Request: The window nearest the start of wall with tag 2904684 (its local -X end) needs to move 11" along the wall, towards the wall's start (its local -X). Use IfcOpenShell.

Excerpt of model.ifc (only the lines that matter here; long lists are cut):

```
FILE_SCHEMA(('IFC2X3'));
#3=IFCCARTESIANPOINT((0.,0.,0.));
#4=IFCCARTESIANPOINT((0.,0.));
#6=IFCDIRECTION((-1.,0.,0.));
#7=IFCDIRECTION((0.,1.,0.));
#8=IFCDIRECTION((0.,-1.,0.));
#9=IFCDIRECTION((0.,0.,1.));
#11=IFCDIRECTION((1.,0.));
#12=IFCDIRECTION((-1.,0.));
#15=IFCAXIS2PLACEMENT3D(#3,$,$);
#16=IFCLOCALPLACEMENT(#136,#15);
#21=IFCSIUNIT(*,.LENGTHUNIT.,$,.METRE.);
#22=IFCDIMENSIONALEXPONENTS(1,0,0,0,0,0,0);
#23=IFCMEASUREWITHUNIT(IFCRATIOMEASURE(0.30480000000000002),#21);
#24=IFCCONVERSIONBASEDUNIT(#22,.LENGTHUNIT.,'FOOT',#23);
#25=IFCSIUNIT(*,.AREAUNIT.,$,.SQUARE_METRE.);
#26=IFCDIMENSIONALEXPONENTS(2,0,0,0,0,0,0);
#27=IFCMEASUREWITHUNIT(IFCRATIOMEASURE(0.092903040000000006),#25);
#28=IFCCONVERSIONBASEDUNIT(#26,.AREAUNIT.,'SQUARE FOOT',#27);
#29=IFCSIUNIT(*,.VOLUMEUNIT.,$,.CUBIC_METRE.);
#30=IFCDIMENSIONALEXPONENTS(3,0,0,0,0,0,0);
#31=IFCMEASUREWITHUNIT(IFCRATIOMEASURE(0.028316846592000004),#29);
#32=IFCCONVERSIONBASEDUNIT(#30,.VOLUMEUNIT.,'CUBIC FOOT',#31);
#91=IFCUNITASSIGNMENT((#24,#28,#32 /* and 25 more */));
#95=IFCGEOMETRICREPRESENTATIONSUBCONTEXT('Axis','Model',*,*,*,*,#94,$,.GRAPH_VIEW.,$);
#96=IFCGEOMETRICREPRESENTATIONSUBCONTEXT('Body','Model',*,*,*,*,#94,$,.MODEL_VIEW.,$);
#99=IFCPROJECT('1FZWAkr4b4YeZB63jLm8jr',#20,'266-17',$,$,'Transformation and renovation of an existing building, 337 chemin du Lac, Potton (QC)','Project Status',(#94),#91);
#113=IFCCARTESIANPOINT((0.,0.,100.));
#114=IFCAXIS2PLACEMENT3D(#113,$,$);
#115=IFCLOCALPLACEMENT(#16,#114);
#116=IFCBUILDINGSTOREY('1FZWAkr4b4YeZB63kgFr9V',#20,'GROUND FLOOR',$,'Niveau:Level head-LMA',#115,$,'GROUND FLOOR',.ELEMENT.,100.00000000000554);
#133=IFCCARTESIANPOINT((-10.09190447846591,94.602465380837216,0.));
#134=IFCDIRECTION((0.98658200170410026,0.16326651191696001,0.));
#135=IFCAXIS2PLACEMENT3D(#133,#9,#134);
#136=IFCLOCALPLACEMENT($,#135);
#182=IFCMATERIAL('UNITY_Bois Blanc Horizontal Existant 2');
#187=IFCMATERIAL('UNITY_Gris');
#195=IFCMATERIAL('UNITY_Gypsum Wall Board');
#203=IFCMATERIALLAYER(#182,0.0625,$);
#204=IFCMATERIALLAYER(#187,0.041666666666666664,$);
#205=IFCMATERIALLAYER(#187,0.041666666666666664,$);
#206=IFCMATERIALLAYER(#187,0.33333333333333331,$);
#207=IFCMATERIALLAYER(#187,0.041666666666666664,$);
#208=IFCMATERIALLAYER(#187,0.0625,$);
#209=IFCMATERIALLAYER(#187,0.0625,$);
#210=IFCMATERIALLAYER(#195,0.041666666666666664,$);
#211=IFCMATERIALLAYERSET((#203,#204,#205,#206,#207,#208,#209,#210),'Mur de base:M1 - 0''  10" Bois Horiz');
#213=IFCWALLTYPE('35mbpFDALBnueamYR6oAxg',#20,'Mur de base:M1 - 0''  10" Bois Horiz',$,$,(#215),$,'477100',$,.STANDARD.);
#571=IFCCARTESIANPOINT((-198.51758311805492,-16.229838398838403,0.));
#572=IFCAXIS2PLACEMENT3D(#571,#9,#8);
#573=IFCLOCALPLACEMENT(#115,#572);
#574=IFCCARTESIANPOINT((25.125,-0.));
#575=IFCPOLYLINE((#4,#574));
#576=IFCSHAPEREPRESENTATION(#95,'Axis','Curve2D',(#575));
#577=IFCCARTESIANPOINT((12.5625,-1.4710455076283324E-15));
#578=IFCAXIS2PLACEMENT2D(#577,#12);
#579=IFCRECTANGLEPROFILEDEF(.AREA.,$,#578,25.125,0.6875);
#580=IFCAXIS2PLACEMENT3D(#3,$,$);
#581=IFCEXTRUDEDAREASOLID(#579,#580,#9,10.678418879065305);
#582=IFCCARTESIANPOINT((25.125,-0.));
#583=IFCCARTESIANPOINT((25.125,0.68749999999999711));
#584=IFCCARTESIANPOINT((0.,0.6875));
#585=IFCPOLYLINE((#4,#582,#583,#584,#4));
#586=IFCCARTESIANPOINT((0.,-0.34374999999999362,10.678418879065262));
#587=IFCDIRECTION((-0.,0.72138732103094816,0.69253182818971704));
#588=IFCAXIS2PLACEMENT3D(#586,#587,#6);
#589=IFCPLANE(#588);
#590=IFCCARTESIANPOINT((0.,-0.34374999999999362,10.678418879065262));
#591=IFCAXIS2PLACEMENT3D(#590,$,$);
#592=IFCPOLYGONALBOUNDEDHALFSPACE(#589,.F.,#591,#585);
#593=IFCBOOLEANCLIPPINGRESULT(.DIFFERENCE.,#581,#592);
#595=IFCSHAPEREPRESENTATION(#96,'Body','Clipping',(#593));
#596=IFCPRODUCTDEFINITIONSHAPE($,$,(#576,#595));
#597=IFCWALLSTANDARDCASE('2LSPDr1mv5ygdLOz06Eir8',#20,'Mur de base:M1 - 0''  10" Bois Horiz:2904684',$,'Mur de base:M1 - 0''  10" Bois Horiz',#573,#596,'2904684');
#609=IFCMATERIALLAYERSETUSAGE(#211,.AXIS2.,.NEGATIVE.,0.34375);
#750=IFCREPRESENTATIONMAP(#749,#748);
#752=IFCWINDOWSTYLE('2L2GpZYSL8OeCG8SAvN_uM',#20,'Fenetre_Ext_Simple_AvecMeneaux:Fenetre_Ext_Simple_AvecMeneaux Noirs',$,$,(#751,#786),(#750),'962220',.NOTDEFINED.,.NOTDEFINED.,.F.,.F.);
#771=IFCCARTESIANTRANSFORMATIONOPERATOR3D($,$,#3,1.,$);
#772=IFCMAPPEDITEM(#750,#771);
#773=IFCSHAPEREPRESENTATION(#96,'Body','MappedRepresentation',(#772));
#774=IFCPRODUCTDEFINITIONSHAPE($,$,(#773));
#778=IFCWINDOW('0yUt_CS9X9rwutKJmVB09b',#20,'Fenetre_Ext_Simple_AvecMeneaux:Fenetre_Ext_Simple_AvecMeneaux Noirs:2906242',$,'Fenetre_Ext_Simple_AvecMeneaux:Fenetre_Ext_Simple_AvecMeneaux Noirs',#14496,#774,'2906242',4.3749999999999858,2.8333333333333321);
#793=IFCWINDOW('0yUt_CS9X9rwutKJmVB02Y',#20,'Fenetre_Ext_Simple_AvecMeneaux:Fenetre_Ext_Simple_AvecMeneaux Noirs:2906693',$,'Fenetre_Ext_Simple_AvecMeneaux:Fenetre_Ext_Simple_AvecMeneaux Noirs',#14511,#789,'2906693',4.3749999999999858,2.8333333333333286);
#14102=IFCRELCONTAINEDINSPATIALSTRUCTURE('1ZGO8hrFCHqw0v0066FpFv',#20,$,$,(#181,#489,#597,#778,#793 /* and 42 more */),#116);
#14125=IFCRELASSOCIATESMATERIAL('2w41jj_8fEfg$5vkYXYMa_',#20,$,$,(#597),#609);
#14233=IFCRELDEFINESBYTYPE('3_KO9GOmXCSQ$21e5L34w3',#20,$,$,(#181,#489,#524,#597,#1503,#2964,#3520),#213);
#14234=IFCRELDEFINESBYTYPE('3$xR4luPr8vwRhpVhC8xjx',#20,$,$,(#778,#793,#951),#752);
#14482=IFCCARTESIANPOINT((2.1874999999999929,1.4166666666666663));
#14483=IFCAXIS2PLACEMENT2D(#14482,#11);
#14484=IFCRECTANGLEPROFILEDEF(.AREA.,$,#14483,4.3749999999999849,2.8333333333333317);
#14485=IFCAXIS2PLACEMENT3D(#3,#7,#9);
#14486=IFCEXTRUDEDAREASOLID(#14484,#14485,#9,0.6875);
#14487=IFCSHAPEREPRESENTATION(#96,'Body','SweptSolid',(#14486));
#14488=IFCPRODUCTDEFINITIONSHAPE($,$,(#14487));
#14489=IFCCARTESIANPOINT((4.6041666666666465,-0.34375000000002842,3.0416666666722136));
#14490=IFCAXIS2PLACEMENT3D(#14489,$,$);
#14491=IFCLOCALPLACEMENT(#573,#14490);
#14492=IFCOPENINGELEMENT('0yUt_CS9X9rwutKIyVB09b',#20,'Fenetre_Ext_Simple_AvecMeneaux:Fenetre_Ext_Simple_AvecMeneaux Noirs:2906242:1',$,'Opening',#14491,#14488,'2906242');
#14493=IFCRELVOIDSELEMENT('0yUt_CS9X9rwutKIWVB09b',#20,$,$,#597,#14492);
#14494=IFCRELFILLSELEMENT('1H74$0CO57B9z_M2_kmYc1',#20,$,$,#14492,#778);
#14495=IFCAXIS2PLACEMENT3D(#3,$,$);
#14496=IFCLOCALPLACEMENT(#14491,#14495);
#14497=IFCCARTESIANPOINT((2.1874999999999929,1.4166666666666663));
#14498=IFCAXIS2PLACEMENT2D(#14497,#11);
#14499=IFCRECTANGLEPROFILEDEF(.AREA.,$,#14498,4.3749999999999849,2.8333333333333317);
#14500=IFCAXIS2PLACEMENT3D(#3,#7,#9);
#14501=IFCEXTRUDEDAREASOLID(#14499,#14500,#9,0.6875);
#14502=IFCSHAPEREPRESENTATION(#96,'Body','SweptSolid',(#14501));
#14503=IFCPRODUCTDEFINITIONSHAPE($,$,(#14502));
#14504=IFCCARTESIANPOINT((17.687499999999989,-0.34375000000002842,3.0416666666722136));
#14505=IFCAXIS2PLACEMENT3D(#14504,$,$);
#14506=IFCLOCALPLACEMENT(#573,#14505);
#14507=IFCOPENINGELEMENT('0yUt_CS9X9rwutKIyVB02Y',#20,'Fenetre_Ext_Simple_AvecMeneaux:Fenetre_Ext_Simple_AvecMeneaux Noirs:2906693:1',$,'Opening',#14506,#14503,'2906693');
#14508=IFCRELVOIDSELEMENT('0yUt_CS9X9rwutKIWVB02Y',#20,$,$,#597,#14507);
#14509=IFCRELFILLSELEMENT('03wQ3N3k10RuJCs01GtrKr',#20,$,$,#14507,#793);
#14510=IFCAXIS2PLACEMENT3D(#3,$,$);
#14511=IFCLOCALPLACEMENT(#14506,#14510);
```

```python
import ifcopenshell
import ifcopenshell.api.geometry
import ifcopenshell.util.placement
import ifcopenshell.util.unit

model = ifcopenshell.open("model.ifc")
unit_scale = ifcopenshell.util.unit.calculate_unit_scale(model)

window = model.by_id(778)
opening = window.FillsVoids[0].RelatingOpeningElement
wall = opening.VoidsElements[0].RelatingBuildingElement

wall_matrix = ifcopenshell.util.placement.get_local_placement(wall.ObjectPlacement)
shift = wall_matrix[:3, 0] * -11 * 0.0254 / unit_scale
before = ifcopenshell.util.placement.get_local_placement(window.ObjectPlacement)[:3, 3].copy()

# The window is placed relative to its opening, so it follows when the opening moves.
matrix = ifcopenshell.util.placement.get_local_placement(opening.ObjectPlacement)
matrix[:3, 3] += shift
ifcopenshell.api.geometry.edit_object_placement(
    model, product=opening, matrix=matrix, is_si=False, should_transform_children=True
)

after = ifcopenshell.util.placement.get_local_placement(window.ObjectPlacement)[:3, 3]
print("window moved by", (after - before).round(3) + 0.0)

model.write("model_edited.ifc")
```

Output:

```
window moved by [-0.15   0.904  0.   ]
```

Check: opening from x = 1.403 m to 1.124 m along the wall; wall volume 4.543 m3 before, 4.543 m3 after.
